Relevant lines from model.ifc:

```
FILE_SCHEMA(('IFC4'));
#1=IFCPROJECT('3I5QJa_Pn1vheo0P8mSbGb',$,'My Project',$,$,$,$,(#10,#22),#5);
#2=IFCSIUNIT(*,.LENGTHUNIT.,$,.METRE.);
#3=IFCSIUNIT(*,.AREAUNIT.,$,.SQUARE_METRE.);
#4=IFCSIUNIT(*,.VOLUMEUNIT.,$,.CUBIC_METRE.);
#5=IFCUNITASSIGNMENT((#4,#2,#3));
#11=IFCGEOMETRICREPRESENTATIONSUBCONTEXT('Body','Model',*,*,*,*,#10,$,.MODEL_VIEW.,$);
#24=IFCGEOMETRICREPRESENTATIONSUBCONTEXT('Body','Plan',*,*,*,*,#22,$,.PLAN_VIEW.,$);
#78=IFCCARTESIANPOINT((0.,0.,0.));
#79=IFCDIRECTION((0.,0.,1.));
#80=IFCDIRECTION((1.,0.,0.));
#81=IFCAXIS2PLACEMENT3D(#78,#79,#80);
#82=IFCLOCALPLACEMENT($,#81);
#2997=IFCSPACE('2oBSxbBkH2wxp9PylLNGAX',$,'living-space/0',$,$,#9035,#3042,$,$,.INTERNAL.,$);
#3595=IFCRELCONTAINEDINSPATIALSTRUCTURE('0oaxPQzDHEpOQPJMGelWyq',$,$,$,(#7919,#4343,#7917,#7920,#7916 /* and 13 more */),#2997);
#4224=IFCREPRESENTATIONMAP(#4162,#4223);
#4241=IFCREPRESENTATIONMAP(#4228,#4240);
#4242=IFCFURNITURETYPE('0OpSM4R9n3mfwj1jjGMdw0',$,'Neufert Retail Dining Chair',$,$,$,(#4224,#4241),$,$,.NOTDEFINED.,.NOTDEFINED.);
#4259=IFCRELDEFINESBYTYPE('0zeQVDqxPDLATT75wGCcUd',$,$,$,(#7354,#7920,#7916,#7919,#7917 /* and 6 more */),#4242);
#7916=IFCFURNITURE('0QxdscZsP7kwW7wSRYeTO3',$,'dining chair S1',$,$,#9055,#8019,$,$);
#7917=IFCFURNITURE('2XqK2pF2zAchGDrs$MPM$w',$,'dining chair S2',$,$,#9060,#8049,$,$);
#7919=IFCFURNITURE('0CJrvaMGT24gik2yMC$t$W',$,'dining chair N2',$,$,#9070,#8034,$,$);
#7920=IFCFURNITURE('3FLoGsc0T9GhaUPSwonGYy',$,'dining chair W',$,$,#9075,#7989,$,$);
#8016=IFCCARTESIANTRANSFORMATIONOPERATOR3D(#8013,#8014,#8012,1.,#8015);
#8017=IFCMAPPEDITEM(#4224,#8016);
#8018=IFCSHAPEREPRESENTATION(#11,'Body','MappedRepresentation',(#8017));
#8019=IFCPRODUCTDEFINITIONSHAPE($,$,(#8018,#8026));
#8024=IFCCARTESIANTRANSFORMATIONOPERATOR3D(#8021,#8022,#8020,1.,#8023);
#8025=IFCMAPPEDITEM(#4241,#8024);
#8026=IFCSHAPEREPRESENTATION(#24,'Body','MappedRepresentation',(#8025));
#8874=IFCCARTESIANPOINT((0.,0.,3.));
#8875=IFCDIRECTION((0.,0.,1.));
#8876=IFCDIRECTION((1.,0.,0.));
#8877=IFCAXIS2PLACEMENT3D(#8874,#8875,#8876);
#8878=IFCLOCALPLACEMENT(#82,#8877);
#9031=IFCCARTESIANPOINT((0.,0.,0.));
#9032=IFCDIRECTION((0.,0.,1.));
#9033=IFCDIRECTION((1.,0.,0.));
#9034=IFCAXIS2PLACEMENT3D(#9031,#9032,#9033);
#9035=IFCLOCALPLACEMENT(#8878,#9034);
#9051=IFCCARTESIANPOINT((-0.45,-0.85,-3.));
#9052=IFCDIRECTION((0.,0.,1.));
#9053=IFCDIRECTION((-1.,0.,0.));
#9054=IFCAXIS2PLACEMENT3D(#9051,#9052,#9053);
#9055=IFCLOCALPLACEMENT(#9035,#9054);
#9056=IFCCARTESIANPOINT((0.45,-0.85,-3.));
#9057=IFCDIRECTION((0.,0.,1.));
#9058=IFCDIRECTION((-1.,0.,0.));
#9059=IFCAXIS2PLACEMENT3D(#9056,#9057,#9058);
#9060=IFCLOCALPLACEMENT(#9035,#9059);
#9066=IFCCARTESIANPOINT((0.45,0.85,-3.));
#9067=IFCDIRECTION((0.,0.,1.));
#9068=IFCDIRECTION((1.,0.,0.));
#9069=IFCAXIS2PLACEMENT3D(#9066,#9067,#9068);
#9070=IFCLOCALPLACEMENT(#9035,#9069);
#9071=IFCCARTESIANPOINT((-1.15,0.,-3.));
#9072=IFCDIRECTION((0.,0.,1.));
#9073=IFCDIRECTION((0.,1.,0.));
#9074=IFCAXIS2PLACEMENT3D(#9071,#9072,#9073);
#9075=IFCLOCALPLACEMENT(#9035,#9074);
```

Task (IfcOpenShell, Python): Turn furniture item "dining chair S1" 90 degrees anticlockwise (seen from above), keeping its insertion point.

```python
import ifcopenshell
import ifcopenshell.api.geometry
import ifcopenshell.util.placement

model = ifcopenshell.open("model.ifc")

item = model.by_guid("0QxdscZsP7kwW7wSRYeTO3")
matrix = ifcopenshell.util.placement.get_local_placement(item.ObjectPlacement)
matrix = matrix @ ifcopenshell.util.placement.rotation(90, "Z")
ifcopenshell.api.geometry.edit_object_placement(model, product=item, matrix=matrix, is_si=False)

print(ifcopenshell.util.placement.get_local_placement(item.ObjectPlacement).round(3) + 0.0)

model.write("model_edited.ifc")
```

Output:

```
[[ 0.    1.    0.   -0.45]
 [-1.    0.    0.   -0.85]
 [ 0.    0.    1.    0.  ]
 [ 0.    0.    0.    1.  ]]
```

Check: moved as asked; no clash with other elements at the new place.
